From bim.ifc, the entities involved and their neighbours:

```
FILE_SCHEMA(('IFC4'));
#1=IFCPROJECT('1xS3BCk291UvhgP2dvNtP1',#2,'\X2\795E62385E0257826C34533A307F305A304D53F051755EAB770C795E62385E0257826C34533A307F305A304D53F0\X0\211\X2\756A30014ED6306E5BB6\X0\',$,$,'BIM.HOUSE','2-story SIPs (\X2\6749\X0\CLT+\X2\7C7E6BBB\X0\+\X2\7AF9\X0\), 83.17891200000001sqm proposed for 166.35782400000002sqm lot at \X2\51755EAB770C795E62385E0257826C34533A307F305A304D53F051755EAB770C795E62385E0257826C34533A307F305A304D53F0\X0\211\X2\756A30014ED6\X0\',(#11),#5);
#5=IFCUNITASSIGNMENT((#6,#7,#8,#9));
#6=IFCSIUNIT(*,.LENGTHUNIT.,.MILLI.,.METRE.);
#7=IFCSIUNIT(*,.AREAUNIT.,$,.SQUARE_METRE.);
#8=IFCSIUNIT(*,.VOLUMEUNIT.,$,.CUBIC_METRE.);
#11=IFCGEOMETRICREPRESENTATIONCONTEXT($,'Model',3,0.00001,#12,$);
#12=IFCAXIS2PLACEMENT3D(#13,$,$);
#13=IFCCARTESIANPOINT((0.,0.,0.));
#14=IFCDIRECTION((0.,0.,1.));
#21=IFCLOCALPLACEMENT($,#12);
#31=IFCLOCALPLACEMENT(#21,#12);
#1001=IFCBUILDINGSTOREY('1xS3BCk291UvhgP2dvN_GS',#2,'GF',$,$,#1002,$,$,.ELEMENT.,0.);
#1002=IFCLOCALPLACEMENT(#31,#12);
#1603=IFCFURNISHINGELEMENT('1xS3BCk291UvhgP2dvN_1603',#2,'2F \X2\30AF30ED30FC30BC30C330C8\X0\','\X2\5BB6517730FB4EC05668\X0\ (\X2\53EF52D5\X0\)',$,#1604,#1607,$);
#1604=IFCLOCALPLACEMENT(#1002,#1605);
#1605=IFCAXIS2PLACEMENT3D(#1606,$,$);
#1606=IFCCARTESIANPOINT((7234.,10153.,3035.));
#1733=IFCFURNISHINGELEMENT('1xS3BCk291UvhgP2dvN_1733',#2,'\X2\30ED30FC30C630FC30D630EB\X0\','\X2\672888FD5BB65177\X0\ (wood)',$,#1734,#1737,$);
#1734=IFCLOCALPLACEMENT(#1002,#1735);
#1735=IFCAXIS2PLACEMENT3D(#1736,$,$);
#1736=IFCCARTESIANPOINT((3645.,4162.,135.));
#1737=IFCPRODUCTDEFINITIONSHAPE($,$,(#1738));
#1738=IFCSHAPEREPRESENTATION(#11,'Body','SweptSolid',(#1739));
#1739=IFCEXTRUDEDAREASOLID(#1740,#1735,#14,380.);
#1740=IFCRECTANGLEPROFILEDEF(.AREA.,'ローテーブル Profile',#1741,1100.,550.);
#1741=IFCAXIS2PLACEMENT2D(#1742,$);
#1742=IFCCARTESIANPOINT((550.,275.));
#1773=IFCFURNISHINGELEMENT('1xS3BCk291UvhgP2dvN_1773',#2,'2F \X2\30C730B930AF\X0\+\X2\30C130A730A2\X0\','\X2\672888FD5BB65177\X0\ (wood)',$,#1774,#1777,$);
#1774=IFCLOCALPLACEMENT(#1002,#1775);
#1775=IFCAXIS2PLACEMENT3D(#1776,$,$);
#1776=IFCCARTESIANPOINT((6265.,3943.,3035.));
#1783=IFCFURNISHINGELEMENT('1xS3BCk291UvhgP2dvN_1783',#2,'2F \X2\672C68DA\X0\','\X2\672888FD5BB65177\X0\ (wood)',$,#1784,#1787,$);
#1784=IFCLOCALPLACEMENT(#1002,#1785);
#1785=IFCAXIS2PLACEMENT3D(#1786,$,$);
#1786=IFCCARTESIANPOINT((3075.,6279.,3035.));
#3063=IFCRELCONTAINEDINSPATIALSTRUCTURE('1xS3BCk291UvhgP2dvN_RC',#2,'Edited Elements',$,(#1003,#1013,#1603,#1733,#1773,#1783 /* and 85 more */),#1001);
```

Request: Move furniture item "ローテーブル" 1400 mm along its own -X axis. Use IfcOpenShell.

```python
import ifcopenshell
import ifcopenshell.api.geometry
import ifcopenshell.util.placement

model = ifcopenshell.open("bim.ifc")

item = model.by_guid("1xS3BCk291UvhgP2dvN_1733")
matrix = ifcopenshell.util.placement.get_local_placement(item.ObjectPlacement)
matrix[:3, 3] -= matrix[:3, 0] * 1400.0
ifcopenshell.api.geometry.edit_object_placement(model, product=item, matrix=matrix, is_si=False)

print(ifcopenshell.util.placement.get_local_placement(item.ObjectPlacement).round(3) + 0.0)

model.write("bim_updated.ifc")
```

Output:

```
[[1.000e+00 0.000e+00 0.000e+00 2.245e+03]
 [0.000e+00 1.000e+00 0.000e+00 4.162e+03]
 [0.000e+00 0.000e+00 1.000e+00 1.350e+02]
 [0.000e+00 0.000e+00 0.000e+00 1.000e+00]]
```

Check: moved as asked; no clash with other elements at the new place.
